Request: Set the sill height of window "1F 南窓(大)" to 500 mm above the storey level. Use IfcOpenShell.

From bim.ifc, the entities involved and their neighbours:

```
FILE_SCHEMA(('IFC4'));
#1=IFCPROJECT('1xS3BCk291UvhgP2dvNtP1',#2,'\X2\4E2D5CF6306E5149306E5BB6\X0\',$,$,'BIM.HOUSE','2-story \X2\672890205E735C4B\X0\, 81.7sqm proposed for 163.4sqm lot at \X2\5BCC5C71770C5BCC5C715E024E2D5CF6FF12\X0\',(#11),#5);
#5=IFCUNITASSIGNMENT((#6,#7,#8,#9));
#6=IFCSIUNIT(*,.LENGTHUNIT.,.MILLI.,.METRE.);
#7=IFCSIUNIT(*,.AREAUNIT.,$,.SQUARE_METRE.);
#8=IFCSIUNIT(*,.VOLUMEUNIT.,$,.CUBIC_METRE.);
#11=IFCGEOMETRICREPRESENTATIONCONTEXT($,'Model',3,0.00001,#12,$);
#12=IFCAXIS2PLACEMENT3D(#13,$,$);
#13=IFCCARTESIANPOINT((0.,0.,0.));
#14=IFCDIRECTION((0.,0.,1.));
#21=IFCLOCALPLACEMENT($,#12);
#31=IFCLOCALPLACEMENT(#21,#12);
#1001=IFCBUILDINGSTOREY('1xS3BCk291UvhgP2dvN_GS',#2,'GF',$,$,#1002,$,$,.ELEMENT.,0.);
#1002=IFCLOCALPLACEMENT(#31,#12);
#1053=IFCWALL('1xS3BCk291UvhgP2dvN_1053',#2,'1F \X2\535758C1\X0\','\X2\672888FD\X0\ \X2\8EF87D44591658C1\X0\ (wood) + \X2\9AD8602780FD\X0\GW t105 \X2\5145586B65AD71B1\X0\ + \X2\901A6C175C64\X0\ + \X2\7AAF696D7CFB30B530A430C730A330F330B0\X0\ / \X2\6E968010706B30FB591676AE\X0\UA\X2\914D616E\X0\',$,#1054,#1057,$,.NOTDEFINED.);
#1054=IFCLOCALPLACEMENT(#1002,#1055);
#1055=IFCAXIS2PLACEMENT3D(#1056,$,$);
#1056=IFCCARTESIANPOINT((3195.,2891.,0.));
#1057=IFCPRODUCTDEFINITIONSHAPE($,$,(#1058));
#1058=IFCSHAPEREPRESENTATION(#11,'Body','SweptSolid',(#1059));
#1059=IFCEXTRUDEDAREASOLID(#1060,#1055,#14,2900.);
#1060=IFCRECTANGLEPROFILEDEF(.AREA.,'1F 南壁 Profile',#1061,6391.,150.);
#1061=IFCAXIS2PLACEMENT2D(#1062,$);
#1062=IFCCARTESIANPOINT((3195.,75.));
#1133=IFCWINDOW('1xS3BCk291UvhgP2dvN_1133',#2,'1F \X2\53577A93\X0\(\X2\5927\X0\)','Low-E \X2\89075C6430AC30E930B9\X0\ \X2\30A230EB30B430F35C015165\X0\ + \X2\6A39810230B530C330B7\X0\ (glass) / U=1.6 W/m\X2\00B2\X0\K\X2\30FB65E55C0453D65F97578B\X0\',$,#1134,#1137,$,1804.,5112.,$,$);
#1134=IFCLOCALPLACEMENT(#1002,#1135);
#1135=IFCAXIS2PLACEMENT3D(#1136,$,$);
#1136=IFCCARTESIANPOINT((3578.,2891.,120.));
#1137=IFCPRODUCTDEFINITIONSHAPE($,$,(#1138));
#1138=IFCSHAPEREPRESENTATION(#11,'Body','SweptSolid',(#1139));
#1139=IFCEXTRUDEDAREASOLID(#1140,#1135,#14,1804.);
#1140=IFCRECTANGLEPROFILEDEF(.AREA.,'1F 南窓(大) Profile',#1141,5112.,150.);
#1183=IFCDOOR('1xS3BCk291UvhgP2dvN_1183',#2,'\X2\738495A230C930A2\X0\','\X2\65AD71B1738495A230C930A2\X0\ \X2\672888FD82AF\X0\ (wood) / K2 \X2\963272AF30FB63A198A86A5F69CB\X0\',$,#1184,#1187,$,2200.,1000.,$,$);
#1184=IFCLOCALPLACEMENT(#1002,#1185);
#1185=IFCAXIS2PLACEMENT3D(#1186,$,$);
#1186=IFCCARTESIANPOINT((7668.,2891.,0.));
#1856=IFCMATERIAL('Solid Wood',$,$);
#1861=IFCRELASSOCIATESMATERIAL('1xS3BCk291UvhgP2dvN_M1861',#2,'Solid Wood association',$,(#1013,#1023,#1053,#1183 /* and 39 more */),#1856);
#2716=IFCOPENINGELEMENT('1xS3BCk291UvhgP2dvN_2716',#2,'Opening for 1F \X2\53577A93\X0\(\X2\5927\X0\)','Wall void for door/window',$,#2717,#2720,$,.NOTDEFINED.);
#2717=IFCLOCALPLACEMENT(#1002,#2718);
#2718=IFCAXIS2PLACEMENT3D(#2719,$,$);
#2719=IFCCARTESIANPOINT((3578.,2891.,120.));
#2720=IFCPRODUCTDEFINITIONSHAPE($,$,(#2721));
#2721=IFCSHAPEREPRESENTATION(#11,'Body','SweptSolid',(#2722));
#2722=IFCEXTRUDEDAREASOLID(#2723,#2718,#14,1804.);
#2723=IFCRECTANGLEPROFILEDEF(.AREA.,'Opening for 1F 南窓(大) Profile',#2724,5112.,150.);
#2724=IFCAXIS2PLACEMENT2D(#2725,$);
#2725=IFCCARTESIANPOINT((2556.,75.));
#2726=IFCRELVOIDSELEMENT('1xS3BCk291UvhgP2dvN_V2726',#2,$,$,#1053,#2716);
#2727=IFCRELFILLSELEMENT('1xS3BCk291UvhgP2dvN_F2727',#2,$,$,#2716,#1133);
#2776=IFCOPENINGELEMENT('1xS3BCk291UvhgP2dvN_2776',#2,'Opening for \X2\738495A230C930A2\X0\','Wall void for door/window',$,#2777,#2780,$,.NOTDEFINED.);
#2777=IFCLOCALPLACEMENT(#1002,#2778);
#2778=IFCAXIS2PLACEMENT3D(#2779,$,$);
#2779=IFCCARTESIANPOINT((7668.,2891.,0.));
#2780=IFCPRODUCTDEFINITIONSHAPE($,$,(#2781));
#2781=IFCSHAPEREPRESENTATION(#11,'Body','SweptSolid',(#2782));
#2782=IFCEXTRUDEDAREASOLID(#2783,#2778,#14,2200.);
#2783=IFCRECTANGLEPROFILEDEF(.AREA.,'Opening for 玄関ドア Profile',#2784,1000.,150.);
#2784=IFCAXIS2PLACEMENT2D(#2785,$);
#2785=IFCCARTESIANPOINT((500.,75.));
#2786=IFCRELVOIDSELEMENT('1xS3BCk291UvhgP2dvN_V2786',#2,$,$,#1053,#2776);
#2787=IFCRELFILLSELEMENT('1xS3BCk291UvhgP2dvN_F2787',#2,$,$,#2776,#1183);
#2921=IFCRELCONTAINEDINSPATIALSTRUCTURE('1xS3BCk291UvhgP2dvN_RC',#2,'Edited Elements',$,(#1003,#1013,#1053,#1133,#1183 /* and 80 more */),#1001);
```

```python
import numpy as np
import ifcopenshell
import ifcopenshell.api.geometry
import ifcopenshell.geom
import ifcopenshell.util.element
import ifcopenshell.util.placement
import ifcopenshell.util.shape
import ifcopenshell.util.unit

model = ifcopenshell.open("bim.ifc")
unit_scale = ifcopenshell.util.unit.calculate_unit_scale(model)

window = model.by_guid("1xS3BCk291UvhgP2dvN_1133")
opening = window.FillsVoids[0].RelatingOpeningElement
storey = ifcopenshell.util.element.get_container(window, ifc_class="IfcBuildingStorey")
level = ifcopenshell.util.placement.get_local_placement(storey.ObjectPlacement)[2, 3]

# The opening's origin need not be at the sill, so measure its lowest point.
shape = ifcopenshell.geom.create_shape(ifcopenshell.geom.settings(), opening)
bottom = ifcopenshell.util.shape.get_shape_bottom_elevation(shape, shape.geometry) / unit_scale
dz = level + 0.5 / unit_scale - bottom

shift = np.array([0.0, 0.0, dz])
# The window is not placed relative to its opening, so move both.
for product in (opening, window):
    matrix = ifcopenshell.util.placement.get_local_placement(product.ObjectPlacement)
    matrix[:3, 3] += shift
    ifcopenshell.api.geometry.edit_object_placement(model, product=product, matrix=matrix, is_si=False)

print(f"moved by {dz * unit_scale:+.3f} m")

model.write("bim-out.ifc")
```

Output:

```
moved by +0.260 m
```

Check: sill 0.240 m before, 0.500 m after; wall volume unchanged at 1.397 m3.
